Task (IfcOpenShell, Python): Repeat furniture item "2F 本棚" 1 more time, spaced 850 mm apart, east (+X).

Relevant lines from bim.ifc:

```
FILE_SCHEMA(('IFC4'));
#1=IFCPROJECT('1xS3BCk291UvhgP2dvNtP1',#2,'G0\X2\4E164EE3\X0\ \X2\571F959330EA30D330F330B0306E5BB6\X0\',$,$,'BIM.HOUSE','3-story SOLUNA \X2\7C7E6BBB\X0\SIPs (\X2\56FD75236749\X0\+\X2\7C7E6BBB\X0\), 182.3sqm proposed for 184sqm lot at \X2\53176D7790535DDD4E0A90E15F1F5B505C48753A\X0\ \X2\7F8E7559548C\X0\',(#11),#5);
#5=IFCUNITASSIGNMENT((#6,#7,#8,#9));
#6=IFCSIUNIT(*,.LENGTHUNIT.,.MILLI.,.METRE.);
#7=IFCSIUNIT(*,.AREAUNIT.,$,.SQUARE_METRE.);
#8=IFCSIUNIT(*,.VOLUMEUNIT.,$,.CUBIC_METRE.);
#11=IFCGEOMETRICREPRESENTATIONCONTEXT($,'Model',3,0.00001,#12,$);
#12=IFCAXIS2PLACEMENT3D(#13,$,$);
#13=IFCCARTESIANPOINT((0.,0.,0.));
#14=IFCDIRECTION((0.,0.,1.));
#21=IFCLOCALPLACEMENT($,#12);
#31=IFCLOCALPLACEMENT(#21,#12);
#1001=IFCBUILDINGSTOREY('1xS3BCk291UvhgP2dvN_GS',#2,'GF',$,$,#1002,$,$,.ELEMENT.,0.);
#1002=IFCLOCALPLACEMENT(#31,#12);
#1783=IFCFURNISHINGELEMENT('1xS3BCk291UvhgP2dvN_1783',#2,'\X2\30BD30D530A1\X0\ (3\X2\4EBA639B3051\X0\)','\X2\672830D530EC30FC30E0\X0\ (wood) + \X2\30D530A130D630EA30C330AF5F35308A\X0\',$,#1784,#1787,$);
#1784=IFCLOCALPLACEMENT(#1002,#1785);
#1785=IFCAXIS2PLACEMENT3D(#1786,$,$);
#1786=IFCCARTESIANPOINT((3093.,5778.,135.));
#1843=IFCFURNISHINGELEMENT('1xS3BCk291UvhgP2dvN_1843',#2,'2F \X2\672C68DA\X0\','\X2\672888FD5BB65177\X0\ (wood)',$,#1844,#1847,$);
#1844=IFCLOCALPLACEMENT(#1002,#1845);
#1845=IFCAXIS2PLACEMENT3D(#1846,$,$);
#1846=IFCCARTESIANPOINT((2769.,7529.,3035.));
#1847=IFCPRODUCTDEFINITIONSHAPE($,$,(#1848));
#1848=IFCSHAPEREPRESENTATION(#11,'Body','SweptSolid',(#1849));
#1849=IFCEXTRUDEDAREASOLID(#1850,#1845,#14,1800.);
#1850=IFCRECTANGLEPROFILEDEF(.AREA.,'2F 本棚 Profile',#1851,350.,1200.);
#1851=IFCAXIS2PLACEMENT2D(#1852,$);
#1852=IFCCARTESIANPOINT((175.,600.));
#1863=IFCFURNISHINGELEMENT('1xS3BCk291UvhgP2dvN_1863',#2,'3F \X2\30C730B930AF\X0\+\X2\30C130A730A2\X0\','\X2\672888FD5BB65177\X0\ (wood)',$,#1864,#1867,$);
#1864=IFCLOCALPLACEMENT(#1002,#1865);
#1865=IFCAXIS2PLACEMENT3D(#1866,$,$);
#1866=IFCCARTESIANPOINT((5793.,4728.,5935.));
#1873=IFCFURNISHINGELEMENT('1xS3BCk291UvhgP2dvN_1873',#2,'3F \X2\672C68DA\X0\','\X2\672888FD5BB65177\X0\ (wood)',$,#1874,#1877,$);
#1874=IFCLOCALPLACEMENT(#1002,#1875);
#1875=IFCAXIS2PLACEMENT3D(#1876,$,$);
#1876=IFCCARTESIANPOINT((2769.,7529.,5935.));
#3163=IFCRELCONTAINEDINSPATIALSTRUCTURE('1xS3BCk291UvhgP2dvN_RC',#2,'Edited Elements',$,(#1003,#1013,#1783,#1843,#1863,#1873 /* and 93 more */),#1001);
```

```python
import numpy as np
import ifcopenshell
import ifcopenshell.api.geometry
import ifcopenshell.api.root
import ifcopenshell.util.element
import ifcopenshell.util.placement

model = ifcopenshell.open("bim.ifc")


def reuse_history(source, copy):
    """copy_class also copies each property set's owner history, people and application; keep the originals."""
    for rel in copy.IsDefinedBy:
        if rel.is_a("IfcRelDefinesByProperties") and (history := rel.RelatingPropertyDefinition.OwnerHistory):
            rel.RelatingPropertyDefinition.OwnerHistory = source.OwnerHistory
            ifcopenshell.util.element.remove_deep2(model, history)


source = model.by_guid("1xS3BCk291UvhgP2dvN_1843")
base = ifcopenshell.util.placement.get_local_placement(source.ObjectPlacement)
step = np.array([1.0, 0.0, 0.0]) * 850.0

for i in range(1, 2):
    copy = ifcopenshell.api.root.copy_class(model, product=source)
    copy.Representation = ifcopenshell.util.element.copy_deep(
        model, source.Representation, exclude=["IfcGeometricRepresentationContext", "IfcRepresentationMap"]
    )
    reuse_history(source, copy)
    matrix = base.copy()
    matrix[:3, 3] += i * step
    print("added at", matrix[:3, 3].round(3) + 0.0)
    ifcopenshell.api.geometry.edit_object_placement(model, product=copy, matrix=matrix, is_si=False)

model.write("bim_v2.ifc")
```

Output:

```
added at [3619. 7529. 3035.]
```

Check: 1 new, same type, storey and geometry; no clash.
